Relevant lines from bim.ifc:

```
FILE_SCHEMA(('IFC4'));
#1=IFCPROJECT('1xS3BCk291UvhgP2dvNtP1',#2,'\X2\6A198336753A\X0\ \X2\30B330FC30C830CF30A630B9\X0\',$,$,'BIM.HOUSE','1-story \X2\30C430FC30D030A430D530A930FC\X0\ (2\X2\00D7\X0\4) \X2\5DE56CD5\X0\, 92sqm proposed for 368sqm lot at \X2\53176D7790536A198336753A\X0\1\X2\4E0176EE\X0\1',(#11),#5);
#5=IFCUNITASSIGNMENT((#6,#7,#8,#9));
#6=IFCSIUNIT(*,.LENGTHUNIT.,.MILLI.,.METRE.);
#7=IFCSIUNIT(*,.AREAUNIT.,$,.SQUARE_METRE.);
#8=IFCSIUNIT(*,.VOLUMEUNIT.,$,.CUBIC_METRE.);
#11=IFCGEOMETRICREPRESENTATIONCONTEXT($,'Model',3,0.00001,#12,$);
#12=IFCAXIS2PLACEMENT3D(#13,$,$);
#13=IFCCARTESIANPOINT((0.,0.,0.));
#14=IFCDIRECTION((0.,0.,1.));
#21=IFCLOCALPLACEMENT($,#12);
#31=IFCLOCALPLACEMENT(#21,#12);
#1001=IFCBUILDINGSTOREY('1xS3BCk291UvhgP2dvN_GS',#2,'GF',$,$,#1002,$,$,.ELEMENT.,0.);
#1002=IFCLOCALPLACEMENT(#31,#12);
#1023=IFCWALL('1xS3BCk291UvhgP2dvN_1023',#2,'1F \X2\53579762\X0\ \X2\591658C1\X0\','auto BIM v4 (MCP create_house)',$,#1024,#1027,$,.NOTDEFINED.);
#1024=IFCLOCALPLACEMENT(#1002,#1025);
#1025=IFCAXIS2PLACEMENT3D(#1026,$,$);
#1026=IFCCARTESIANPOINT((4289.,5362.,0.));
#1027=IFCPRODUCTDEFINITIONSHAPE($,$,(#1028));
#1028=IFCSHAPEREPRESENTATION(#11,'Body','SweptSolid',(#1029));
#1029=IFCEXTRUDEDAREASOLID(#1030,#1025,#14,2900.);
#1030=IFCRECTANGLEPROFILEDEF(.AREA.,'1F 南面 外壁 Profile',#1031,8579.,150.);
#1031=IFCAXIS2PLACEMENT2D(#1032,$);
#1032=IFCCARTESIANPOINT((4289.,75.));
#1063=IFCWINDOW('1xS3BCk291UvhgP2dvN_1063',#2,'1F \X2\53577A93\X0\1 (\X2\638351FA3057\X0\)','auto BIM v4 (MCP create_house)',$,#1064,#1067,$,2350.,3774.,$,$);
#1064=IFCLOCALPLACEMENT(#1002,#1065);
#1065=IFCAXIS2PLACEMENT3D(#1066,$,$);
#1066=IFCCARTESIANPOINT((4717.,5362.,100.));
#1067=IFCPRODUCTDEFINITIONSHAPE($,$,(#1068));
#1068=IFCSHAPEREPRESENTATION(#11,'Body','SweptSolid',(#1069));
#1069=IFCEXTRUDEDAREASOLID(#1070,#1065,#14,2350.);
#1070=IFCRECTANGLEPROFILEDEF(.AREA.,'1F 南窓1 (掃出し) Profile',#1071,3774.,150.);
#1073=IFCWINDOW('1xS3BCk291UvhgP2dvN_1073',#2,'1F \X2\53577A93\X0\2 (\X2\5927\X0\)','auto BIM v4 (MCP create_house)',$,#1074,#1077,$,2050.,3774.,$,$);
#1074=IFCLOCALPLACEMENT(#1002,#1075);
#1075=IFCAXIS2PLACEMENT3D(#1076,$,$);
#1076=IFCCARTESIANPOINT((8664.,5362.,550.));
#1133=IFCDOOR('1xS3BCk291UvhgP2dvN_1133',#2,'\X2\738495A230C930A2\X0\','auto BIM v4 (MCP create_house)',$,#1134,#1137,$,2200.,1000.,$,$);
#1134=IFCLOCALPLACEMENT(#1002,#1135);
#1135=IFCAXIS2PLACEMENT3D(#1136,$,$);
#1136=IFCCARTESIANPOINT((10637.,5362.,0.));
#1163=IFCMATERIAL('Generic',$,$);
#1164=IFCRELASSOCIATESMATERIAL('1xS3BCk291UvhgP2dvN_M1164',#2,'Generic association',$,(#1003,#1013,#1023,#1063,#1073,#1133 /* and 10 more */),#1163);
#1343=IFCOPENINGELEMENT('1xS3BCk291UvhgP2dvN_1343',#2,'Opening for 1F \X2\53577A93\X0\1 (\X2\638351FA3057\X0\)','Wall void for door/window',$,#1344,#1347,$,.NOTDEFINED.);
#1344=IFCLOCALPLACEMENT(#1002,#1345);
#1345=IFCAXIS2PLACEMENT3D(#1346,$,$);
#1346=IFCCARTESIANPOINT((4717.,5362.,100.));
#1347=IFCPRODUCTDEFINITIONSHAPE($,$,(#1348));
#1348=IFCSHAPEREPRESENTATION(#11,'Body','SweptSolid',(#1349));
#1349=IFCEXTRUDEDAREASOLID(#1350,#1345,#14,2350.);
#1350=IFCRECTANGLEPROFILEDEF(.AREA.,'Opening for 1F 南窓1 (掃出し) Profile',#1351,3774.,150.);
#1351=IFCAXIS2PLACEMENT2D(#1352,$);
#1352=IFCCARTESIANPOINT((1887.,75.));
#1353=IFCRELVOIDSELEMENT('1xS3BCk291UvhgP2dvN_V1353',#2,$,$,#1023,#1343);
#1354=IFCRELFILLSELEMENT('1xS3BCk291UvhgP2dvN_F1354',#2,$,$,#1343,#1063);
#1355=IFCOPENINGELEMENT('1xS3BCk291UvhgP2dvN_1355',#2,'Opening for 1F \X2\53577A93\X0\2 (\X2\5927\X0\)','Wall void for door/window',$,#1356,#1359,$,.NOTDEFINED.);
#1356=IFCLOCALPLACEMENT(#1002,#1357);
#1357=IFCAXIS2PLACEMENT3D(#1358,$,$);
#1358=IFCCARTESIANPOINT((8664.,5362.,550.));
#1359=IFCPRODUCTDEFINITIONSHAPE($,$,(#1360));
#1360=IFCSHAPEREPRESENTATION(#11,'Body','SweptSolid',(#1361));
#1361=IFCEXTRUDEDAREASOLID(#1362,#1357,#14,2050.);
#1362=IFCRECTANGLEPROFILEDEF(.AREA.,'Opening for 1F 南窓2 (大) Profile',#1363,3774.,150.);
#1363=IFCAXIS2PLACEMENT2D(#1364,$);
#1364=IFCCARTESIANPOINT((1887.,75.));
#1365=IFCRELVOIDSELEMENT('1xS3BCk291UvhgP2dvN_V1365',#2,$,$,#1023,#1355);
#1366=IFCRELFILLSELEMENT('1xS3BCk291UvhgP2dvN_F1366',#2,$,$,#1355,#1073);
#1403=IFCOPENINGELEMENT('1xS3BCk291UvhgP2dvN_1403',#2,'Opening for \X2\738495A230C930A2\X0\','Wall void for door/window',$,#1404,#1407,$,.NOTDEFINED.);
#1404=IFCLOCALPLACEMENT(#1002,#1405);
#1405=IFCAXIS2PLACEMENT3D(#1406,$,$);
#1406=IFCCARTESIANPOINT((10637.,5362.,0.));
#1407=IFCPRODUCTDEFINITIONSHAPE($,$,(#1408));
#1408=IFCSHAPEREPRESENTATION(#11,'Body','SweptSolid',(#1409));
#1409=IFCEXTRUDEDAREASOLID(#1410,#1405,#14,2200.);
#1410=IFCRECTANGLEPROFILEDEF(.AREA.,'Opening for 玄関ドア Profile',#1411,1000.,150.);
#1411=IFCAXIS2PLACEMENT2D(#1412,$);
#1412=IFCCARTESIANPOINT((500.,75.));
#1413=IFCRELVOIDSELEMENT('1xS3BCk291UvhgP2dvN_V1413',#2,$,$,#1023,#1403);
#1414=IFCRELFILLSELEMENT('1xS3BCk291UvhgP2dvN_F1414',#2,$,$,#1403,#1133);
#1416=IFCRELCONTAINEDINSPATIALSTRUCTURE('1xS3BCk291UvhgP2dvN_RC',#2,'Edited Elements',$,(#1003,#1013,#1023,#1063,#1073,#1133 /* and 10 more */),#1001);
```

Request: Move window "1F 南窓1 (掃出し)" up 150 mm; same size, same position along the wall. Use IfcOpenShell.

```python
import numpy as np
import ifcopenshell
import ifcopenshell.api.geometry
import ifcopenshell.util.placement
import ifcopenshell.util.unit

model = ifcopenshell.open("bim.ifc")
unit_scale = ifcopenshell.util.unit.calculate_unit_scale(model)

window = model.by_id(1063)
opening = window.FillsVoids[0].RelatingOpeningElement
dz = 0.15 / unit_scale

shift = np.array([0.0, 0.0, dz])
# The window is not placed relative to its opening, so move both.
for product in (opening, window):
    matrix = ifcopenshell.util.placement.get_local_placement(product.ObjectPlacement)
    matrix[:3, 3] += shift
    ifcopenshell.api.geometry.edit_object_placement(model, product=product, matrix=matrix, is_si=False)

print(f"moved by {dz * unit_scale:+.3f} m")

model.write("bim_v2.ifc")
```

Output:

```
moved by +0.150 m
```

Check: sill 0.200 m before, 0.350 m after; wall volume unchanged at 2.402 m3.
